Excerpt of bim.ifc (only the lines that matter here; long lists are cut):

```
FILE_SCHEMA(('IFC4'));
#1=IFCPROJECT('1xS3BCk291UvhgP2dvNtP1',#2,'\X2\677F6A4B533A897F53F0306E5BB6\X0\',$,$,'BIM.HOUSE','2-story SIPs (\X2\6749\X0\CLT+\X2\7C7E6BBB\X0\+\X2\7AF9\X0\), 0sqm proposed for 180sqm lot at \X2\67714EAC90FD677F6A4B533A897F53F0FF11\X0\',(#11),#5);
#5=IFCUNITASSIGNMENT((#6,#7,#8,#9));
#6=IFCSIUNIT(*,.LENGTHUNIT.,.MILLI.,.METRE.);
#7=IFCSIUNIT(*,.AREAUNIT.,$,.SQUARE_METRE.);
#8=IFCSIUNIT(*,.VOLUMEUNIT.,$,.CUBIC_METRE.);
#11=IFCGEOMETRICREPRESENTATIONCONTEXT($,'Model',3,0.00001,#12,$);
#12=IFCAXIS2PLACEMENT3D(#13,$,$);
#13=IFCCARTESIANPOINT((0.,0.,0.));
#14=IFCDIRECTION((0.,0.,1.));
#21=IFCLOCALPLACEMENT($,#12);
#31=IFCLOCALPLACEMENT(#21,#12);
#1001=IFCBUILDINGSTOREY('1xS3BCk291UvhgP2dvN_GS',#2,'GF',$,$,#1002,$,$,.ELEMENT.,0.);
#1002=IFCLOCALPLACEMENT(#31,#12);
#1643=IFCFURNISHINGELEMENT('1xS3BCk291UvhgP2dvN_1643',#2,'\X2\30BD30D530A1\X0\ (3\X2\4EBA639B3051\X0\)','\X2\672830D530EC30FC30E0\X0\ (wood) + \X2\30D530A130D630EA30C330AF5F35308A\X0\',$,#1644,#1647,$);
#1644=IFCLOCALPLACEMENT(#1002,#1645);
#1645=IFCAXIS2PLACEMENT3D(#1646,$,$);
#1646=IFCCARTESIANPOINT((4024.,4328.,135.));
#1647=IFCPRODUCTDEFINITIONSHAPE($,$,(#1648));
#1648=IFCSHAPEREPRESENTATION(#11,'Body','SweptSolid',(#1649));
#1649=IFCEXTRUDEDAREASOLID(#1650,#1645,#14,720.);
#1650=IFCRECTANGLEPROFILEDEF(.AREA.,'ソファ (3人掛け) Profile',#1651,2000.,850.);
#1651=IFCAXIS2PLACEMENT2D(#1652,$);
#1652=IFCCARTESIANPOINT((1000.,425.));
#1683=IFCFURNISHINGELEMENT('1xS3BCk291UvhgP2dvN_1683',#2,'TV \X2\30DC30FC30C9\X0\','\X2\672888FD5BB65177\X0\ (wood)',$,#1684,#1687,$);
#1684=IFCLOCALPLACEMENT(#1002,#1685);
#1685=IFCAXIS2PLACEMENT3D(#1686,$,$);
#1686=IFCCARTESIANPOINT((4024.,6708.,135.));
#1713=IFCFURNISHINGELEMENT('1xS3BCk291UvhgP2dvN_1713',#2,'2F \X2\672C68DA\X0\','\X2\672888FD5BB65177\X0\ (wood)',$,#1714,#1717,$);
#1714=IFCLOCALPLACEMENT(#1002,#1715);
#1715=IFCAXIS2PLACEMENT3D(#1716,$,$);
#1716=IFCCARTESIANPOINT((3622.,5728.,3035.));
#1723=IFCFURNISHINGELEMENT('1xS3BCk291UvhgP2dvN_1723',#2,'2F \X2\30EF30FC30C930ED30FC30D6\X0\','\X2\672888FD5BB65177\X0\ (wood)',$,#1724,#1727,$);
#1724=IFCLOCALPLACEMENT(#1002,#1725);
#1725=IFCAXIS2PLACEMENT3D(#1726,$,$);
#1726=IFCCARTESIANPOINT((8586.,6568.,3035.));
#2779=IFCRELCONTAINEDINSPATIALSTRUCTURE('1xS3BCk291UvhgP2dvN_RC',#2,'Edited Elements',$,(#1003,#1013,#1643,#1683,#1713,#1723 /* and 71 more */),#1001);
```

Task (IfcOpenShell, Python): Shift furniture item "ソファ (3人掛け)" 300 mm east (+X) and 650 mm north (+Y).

```python
import ifcopenshell
import ifcopenshell.api.geometry
import ifcopenshell.util.placement
import ifcopenshell.util.unit

model = ifcopenshell.open("bim.ifc")
unit_scale = ifcopenshell.util.unit.calculate_unit_scale(model)

item = model.by_guid("1xS3BCk291UvhgP2dvN_1643")
matrix = ifcopenshell.util.placement.get_local_placement(item.ObjectPlacement)
matrix[0, 3] += 0.3 / unit_scale
matrix[1, 3] += 0.65 / unit_scale
ifcopenshell.api.geometry.edit_object_placement(model, product=item, matrix=matrix, is_si=False)

print(ifcopenshell.util.placement.get_local_placement(item.ObjectPlacement).round(3) + 0.0)

model.write("bim_updated.ifc")
```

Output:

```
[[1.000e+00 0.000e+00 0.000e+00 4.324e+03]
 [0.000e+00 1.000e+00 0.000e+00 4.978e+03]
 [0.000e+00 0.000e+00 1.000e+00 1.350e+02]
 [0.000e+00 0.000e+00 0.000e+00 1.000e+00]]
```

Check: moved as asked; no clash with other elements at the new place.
